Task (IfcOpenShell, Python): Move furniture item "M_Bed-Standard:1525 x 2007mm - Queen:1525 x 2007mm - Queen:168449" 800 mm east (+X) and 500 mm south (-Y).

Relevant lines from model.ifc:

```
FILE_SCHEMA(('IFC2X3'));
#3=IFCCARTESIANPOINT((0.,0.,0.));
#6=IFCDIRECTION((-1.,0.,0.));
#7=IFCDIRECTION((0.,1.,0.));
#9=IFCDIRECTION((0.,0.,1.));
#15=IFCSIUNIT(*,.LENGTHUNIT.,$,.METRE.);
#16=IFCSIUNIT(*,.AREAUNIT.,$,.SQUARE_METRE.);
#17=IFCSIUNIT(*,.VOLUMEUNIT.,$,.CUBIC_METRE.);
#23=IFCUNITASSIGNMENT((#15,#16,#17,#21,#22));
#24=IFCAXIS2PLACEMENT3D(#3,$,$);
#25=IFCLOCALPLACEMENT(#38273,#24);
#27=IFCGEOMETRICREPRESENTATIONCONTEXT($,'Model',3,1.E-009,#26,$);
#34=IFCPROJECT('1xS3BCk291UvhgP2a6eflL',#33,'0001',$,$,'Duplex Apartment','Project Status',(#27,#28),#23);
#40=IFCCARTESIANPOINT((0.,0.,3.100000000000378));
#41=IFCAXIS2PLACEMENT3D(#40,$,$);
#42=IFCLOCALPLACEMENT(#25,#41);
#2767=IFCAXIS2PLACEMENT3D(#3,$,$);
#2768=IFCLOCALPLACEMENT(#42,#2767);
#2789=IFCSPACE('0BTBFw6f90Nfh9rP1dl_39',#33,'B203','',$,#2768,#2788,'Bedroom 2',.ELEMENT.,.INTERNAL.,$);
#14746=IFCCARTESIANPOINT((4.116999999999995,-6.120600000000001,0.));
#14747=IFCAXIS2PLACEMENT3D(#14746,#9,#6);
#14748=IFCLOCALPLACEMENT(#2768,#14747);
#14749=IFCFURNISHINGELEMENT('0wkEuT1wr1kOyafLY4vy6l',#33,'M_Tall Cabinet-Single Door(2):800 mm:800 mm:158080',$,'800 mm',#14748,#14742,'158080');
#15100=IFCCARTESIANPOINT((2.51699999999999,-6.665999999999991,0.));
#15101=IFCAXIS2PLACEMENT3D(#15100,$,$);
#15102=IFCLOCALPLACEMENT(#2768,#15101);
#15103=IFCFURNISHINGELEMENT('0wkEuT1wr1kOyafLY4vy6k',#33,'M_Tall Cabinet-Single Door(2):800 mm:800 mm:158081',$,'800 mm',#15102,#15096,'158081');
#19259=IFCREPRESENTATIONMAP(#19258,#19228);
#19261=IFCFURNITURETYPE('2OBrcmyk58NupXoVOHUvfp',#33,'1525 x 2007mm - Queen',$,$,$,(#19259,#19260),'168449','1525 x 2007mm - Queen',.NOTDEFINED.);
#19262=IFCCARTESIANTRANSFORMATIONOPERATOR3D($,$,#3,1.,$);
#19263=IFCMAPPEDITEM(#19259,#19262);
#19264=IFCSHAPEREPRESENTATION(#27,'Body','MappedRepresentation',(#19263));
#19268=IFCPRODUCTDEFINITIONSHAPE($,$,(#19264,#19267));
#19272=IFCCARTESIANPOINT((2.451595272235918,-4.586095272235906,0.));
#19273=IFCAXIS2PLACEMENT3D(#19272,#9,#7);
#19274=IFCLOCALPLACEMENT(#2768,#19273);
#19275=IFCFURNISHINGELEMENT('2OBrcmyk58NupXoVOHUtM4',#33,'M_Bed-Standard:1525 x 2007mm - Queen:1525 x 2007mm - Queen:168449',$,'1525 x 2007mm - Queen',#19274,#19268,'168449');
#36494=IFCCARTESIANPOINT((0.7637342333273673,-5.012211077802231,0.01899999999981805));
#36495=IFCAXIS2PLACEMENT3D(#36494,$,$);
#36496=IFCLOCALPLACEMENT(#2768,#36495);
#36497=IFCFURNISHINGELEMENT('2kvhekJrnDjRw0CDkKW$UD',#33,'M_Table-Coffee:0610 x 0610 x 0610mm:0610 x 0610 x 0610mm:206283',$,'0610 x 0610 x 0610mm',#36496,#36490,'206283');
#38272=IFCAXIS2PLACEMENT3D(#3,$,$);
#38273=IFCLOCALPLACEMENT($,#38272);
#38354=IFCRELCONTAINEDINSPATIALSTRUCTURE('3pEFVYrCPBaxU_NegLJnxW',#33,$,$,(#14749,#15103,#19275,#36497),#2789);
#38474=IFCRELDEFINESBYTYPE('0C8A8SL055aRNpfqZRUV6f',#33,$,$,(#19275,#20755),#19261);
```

```python
import ifcopenshell
import ifcopenshell.api.geometry
import ifcopenshell.util.placement

model = ifcopenshell.open("model.ifc")

item = model.by_guid("2OBrcmyk58NupXoVOHUtM4")
matrix = ifcopenshell.util.placement.get_local_placement(item.ObjectPlacement)
matrix[0, 3] += 0.8
matrix[1, 3] -= 0.5
ifcopenshell.api.geometry.edit_object_placement(model, product=item, matrix=matrix, is_si=False)

print(ifcopenshell.util.placement.get_local_placement(item.ObjectPlacement).round(3) + 0.0)

model.write("model_rev.ifc")
```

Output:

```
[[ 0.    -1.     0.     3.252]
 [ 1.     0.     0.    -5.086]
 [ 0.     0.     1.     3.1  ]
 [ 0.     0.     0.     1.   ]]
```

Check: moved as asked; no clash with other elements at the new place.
